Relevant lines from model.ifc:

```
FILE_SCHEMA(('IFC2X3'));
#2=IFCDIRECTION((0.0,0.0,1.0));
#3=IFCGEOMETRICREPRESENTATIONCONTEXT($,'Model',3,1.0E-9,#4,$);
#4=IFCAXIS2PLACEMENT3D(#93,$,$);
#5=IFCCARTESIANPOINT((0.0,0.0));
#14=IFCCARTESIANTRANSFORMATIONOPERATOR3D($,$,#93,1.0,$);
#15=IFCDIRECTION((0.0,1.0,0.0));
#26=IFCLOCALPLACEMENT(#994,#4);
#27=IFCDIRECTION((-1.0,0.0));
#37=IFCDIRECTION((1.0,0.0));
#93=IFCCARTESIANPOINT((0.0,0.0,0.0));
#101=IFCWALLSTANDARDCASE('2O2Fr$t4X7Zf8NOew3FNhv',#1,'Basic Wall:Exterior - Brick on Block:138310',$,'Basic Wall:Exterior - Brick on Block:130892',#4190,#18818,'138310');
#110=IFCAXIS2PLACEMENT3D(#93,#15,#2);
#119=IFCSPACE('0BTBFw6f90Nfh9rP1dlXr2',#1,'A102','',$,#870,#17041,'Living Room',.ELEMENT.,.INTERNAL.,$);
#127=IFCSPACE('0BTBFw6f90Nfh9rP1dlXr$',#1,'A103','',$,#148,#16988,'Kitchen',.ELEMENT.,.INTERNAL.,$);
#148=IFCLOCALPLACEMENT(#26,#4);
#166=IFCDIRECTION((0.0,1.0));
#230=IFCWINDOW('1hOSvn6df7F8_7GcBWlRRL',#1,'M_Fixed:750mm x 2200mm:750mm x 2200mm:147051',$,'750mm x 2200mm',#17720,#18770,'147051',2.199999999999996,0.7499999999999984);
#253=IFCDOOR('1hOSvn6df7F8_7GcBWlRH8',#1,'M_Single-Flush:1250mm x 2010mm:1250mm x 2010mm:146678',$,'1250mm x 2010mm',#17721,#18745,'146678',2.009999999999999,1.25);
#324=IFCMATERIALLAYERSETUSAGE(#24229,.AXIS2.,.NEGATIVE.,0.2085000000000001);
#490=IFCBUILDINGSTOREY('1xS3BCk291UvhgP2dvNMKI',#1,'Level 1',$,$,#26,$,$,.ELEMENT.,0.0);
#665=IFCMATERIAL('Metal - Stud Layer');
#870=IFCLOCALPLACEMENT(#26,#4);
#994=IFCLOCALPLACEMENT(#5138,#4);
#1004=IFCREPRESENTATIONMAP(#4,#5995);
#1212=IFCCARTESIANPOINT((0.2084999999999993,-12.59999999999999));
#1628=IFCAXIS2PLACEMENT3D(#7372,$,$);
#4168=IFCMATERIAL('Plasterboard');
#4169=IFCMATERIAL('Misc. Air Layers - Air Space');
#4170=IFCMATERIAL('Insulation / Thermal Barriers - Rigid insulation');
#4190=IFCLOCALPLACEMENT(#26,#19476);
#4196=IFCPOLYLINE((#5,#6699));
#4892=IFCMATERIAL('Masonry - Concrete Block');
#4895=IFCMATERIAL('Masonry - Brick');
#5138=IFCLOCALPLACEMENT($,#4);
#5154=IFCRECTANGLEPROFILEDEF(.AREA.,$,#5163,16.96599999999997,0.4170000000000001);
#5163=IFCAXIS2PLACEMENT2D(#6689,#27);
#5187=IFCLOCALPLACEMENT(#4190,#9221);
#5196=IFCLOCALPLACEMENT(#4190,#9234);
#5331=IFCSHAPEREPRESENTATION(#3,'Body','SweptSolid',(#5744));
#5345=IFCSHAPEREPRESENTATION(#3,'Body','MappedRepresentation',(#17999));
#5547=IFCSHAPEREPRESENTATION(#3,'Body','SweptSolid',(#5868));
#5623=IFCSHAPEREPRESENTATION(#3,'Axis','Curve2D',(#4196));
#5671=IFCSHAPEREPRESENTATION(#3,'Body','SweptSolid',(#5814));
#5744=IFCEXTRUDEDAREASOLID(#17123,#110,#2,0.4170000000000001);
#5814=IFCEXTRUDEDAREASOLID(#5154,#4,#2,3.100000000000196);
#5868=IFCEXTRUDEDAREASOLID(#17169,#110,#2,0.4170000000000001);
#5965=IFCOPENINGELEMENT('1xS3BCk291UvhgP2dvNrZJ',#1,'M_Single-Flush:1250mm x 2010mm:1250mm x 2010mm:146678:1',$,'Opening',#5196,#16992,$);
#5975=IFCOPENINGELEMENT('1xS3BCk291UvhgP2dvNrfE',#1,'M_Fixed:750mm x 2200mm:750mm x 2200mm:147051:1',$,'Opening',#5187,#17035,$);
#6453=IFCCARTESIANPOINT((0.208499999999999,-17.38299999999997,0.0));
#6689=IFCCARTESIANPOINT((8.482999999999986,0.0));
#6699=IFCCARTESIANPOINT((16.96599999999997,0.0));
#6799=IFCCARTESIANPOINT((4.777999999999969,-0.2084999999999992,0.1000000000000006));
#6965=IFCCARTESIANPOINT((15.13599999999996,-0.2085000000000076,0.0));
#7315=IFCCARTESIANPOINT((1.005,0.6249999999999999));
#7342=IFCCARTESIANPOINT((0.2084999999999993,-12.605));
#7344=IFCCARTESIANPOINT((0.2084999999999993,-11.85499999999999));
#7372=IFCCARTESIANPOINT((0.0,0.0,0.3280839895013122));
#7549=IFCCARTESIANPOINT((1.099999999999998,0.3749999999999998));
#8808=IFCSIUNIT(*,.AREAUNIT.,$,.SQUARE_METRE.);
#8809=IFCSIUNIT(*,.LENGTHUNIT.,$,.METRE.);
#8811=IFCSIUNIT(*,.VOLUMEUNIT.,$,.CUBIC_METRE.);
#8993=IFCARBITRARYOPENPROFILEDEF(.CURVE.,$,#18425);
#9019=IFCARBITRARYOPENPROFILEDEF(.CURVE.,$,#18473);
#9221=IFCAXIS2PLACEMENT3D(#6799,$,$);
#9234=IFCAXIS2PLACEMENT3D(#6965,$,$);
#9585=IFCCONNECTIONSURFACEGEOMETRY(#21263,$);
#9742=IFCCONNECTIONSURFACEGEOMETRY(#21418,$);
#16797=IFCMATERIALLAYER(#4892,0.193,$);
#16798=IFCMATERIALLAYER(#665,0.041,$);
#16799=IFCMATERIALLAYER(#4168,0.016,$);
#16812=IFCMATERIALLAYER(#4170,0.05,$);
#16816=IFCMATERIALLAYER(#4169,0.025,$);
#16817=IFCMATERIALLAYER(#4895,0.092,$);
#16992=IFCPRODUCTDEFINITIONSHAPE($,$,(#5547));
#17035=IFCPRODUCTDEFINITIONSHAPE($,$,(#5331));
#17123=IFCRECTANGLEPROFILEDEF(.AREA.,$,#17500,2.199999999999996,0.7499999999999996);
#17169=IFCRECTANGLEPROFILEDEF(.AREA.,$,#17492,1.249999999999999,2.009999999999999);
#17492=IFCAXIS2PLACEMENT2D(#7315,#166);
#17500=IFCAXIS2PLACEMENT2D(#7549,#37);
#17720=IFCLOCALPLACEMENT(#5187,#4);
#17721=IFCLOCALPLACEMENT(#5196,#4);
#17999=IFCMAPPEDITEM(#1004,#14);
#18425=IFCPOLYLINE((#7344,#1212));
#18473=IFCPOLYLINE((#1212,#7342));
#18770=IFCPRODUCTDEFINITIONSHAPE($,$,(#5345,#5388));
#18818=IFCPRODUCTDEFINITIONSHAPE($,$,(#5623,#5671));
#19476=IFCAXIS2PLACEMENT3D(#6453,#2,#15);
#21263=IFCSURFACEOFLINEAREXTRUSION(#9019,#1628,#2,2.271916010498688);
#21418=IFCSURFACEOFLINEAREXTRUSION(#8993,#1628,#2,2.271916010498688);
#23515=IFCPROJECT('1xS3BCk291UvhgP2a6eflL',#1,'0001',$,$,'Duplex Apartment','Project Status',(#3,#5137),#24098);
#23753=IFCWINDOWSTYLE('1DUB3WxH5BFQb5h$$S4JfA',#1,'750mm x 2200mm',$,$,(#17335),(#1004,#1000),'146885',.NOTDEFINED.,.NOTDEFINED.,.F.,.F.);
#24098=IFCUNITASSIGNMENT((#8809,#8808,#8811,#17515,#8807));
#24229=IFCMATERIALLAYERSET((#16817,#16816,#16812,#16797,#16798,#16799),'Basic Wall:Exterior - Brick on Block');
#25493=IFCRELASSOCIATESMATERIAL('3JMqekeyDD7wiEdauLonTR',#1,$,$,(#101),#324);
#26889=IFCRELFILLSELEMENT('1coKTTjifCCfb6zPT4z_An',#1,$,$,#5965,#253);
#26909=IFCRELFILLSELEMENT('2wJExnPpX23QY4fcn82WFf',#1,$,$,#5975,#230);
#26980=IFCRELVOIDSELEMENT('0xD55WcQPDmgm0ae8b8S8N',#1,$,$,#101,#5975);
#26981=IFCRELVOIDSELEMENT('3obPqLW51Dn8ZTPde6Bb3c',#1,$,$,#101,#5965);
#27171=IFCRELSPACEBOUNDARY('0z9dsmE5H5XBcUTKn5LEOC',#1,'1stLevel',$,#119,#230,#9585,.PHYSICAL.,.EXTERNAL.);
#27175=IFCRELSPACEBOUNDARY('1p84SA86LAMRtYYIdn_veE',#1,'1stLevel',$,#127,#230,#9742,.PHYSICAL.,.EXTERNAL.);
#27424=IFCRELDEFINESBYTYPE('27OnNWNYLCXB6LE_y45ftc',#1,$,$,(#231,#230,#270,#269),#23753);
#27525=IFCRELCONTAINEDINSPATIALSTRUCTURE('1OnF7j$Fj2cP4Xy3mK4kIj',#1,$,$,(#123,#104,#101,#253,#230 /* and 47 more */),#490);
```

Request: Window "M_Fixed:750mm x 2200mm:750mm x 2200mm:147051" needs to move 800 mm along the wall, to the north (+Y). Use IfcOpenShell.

```python
import numpy as np
import ifcopenshell
import ifcopenshell.api.geometry
import ifcopenshell.util.placement
import ifcopenshell.util.unit

model = ifcopenshell.open("model.ifc")
unit_scale = ifcopenshell.util.unit.calculate_unit_scale(model)

window = model.by_id(230)
opening = window.FillsVoids[0].RelatingOpeningElement
wall = opening.VoidsElements[0].RelatingBuildingElement

wall_matrix = ifcopenshell.util.placement.get_local_placement(wall.ObjectPlacement)
shift = wall_matrix[:3, 0] * 0.8 / unit_scale
before = ifcopenshell.util.placement.get_local_placement(window.ObjectPlacement)[:3, 3].copy()

# The window is placed relative to its opening, so it follows when the opening moves.
matrix = ifcopenshell.util.placement.get_local_placement(opening.ObjectPlacement)
matrix[:3, 3] += shift
ifcopenshell.api.geometry.edit_object_placement(
    model, product=opening, matrix=matrix, is_si=False, should_transform_children=True
)

# Space boundary surfaces are stored in each space's coordinates; move them too.
for rel in window.ProvidesBoundaries:
    if not rel.ConnectionGeometry:
        continue
    surface = rel.ConnectionGeometry.SurfaceOnRelatingElement
    space_matrix = ifcopenshell.util.placement.get_local_placement(rel.RelatingSpace.ObjectPlacement)
    point = np.array(surface.Position.Location.Coordinates) + space_matrix[:3, :3].T @ shift
    surface.Position = model.createIfcAxis2Placement3D(
        model.createIfcCartesianPoint(point.tolist()), surface.Position.Axis, surface.Position.RefDirection
    )

after = ifcopenshell.util.placement.get_local_placement(window.ObjectPlacement)[:3, 3]
print("window moved by", (after - before).round(3) + 0.0)

model.write("model-out.ifc")
```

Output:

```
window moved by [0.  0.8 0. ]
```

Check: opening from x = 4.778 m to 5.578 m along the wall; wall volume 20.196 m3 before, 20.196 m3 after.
